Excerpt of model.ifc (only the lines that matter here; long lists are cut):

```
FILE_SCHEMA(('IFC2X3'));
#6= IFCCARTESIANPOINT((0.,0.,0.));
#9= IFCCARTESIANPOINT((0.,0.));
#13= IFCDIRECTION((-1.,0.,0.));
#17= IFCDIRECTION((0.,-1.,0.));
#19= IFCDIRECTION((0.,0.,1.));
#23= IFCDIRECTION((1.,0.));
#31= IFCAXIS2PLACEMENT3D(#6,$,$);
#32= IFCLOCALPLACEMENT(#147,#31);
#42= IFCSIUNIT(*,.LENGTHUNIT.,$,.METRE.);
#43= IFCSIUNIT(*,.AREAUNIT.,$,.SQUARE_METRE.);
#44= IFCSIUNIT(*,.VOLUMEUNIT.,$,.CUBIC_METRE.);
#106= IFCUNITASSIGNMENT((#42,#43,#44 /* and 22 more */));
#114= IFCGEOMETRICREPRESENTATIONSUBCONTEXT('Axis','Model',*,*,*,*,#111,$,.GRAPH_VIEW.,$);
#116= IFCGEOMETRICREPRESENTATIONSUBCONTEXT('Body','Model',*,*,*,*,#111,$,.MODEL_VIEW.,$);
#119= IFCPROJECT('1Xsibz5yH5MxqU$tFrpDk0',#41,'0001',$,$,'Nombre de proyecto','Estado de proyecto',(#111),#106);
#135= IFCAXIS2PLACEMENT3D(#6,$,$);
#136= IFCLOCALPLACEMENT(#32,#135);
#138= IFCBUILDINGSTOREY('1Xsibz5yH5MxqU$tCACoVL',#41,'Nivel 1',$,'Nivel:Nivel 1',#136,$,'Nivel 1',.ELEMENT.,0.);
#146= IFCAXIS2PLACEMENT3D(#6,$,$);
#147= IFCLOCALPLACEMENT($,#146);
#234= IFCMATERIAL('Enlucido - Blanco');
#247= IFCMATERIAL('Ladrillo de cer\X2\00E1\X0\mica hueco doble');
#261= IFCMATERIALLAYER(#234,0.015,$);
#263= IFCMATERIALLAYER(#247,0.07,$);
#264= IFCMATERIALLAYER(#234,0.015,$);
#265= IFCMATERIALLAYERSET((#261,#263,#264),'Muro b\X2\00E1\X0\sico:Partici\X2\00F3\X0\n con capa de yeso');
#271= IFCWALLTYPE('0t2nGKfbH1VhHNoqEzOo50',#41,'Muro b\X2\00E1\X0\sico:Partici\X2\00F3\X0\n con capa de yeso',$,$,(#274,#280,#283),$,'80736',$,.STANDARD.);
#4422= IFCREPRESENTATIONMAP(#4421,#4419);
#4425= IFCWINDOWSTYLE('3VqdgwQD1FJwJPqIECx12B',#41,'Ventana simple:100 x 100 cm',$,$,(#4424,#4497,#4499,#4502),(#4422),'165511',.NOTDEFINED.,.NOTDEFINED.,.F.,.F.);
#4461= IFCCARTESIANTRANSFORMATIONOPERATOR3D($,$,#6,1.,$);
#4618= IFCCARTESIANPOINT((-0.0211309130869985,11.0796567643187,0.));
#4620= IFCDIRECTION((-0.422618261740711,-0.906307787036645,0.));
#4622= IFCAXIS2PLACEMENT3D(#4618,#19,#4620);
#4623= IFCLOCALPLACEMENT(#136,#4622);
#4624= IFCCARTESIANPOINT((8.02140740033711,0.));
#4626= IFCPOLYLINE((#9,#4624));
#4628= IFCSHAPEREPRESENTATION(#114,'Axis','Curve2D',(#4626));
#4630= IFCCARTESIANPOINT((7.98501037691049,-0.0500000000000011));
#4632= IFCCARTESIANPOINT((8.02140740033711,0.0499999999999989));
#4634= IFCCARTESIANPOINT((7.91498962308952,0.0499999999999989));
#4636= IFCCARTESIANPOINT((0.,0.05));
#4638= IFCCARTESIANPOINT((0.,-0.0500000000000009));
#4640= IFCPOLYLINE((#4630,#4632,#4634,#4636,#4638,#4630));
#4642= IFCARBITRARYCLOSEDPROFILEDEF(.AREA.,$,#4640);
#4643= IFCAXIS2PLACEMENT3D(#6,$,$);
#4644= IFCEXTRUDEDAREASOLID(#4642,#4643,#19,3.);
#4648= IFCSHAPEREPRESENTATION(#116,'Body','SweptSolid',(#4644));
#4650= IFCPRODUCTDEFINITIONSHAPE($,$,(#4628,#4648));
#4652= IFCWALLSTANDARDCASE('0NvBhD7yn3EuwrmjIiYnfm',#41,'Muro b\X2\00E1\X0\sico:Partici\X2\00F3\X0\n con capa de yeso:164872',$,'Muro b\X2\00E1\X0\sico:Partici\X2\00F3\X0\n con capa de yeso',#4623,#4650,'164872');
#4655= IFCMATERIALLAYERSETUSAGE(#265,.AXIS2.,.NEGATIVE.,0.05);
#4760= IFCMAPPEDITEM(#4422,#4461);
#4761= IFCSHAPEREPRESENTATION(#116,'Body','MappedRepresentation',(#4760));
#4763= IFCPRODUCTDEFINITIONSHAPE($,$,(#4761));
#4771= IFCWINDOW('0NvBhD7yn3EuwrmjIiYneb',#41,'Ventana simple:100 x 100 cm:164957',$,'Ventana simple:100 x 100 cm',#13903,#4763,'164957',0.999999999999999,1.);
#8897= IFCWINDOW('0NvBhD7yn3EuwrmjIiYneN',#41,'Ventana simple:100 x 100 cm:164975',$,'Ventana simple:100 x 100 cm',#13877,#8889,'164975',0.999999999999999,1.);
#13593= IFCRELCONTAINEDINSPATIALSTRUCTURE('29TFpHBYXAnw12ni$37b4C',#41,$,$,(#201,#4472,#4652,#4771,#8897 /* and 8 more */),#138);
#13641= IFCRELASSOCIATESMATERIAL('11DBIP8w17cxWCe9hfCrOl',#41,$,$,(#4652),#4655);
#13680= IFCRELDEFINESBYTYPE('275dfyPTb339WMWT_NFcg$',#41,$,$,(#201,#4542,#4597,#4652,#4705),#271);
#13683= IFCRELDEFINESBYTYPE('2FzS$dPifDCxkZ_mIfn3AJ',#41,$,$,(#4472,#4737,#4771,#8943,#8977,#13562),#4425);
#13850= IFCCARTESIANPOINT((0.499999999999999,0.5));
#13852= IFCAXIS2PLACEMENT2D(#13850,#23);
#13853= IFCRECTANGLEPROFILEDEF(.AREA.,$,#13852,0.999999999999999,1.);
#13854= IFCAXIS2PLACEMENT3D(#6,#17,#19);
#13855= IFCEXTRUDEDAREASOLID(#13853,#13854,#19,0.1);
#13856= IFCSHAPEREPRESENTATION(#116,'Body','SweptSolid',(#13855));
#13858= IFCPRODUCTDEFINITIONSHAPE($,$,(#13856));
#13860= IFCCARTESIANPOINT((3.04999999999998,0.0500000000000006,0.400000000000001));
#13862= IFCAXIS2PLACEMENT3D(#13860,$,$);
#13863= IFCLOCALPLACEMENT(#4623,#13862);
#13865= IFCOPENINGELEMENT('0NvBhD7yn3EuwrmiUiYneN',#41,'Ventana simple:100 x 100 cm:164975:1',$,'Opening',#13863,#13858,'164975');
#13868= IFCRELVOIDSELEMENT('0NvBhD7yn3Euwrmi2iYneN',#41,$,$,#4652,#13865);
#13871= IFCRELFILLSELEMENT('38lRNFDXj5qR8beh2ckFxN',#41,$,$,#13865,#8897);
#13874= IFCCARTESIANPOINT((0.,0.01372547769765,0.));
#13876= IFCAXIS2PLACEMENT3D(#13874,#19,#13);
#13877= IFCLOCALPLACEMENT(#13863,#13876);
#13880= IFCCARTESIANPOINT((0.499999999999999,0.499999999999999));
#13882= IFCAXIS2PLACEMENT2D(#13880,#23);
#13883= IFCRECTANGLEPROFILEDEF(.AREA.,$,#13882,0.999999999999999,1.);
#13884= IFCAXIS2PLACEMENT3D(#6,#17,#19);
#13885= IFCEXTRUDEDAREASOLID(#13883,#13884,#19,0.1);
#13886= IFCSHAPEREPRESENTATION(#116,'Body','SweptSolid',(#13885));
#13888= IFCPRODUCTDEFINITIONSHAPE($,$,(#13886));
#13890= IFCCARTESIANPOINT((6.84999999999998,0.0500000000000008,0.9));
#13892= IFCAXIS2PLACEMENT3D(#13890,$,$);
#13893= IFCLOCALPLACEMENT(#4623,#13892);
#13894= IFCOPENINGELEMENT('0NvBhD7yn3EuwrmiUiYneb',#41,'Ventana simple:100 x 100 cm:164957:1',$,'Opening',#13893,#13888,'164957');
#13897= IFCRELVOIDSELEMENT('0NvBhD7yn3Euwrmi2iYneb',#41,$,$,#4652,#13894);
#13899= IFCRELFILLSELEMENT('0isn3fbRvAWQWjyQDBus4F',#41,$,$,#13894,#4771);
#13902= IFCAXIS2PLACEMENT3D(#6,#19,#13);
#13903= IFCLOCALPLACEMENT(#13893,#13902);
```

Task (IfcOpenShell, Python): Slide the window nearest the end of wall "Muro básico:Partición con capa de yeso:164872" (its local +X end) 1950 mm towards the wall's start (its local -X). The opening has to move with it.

```python
import ifcopenshell
import ifcopenshell.api.geometry
import ifcopenshell.util.placement

model = ifcopenshell.open("model.ifc")

window = model.by_id(4771)
opening = window.FillsVoids[0].RelatingOpeningElement
wall = opening.VoidsElements[0].RelatingBuildingElement

wall_matrix = ifcopenshell.util.placement.get_local_placement(wall.ObjectPlacement)
shift = wall_matrix[:3, 0] * -1.95
before = ifcopenshell.util.placement.get_local_placement(window.ObjectPlacement)[:3, 3].copy()

# The window is placed relative to its opening, so it follows when the opening moves.
matrix = ifcopenshell.util.placement.get_local_placement(opening.ObjectPlacement)
matrix[:3, 3] += shift
ifcopenshell.api.geometry.edit_object_placement(
    model, product=opening, matrix=matrix, is_si=False, should_transform_children=True
)

after = ifcopenshell.util.placement.get_local_placement(window.ObjectPlacement)[:3, 3]
print("window moved by", (after - before).round(3) + 0.0)

model.write("model-out.ifc")
```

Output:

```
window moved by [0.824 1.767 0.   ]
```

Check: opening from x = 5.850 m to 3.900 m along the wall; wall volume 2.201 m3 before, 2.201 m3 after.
